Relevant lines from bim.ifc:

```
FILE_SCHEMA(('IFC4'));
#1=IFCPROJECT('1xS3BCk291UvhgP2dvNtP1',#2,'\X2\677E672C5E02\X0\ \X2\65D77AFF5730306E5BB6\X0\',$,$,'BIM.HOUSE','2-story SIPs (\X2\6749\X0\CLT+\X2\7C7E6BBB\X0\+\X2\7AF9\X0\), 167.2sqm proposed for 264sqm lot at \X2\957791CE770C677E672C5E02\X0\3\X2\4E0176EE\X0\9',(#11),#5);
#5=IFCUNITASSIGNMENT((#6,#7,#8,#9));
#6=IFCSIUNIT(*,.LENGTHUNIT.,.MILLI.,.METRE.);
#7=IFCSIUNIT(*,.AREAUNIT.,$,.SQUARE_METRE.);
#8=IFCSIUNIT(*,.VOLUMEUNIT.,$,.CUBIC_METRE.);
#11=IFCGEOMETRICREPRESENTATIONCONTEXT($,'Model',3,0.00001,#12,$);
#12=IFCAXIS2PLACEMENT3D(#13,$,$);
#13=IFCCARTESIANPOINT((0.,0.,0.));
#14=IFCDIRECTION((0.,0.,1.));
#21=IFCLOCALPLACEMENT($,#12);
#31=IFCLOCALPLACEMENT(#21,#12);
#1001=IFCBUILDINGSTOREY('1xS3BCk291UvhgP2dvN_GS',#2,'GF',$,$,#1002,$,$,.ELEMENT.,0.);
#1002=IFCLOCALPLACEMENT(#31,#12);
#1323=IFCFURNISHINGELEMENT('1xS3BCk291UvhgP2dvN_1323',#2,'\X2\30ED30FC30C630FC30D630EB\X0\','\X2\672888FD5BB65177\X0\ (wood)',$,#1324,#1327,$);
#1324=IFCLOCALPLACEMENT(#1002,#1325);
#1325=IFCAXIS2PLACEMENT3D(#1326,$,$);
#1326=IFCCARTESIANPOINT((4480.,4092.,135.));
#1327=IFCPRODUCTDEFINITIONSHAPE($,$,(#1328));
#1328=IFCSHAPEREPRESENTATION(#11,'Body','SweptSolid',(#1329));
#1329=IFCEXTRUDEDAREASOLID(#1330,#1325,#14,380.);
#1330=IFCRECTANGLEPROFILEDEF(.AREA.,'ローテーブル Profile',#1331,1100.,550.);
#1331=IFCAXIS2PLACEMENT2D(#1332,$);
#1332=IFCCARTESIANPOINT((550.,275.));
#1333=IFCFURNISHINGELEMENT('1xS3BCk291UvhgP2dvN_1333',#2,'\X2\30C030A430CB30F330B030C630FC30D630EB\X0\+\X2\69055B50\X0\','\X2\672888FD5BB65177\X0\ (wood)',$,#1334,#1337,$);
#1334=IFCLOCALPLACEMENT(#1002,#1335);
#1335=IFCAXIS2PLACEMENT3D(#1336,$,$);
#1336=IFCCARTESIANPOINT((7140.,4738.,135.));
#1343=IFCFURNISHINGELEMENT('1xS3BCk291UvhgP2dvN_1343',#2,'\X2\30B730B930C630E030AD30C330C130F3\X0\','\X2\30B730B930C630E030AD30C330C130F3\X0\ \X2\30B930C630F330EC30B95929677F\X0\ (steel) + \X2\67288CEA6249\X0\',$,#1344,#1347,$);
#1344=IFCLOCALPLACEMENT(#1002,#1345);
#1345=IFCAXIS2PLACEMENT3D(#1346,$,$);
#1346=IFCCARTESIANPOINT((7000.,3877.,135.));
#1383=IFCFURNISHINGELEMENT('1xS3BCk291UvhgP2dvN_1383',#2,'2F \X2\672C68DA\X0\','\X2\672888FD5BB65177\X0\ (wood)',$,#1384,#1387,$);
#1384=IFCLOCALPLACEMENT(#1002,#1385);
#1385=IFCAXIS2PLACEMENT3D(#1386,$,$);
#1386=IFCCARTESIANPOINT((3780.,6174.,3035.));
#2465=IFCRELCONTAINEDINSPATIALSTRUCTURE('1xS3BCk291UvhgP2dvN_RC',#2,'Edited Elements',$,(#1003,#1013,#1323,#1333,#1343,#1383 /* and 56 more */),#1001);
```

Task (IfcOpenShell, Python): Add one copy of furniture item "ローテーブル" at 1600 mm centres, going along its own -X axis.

```python
import ifcopenshell
import ifcopenshell.api.geometry
import ifcopenshell.api.root
import ifcopenshell.util.element
import ifcopenshell.util.placement
import ifcopenshell.util.unit

model = ifcopenshell.open("bim.ifc")
unit_scale = ifcopenshell.util.unit.calculate_unit_scale(model)


def reuse_history(source, copy):
    """copy_class also copies each property set's owner history, people and application; keep the originals."""
    for rel in copy.IsDefinedBy:
        if rel.is_a("IfcRelDefinesByProperties") and (history := rel.RelatingPropertyDefinition.OwnerHistory):
            rel.RelatingPropertyDefinition.OwnerHistory = source.OwnerHistory
            ifcopenshell.util.element.remove_deep2(model, history)


source = model.by_guid("1xS3BCk291UvhgP2dvN_1323")
base = ifcopenshell.util.placement.get_local_placement(source.ObjectPlacement)
step = -base[:3, 0] * 1.6 / unit_scale

for i in range(1, 2):
    copy = ifcopenshell.api.root.copy_class(model, product=source)
    copy.Representation = ifcopenshell.util.element.copy_deep(
        model, source.Representation, exclude=["IfcGeometricRepresentationContext", "IfcRepresentationMap"]
    )
    reuse_history(source, copy)
    matrix = base.copy()
    matrix[:3, 3] += i * step
    print("added at", matrix[:3, 3].round(3) + 0.0)
    ifcopenshell.api.geometry.edit_object_placement(model, product=copy, matrix=matrix, is_si=False)

model.write("bim_rev.ifc")
```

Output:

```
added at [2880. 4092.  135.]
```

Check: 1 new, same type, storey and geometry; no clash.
